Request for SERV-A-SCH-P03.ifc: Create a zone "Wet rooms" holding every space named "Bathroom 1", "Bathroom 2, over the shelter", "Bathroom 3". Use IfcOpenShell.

First a look at what the model holds.

```python
import ifcopenshell

model = ifcopenshell.open("SERV-A-SCH-P03.ifc")
print(model.schema)
seen = {}
for space in model.by_type("IfcSpace"):
    seen[space.LongName] = seen.get(space.LongName, 0) + 1
for name, count in sorted(seen.items(), key=str):
    print(count, "x", name)
print("zones:", [z.Name for z in model.by_type("IfcZone")][:20])
```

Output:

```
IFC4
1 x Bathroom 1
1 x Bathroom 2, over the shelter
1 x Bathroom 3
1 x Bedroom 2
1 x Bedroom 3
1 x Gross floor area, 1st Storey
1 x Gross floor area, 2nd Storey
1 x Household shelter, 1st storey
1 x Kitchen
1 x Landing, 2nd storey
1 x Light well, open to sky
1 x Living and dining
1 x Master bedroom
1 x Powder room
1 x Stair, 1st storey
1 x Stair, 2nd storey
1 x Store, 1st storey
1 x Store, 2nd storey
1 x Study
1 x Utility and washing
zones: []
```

```python
import ifcopenshell
import ifcopenshell.api.group
import ifcopenshell.api.root

model = ifcopenshell.open("SERV-A-SCH-P03.ifc")

names = {"Bathroom 1", "Bathroom 2, over the shelter", "Bathroom 3"}
spaces = [s for s in model.by_type("IfcSpace") if s.LongName in names]

zone = ifcopenshell.api.root.create_entity(model, ifc_class="IfcZone", name="Wet rooms")
ifcopenshell.api.group.assign_group(model, products=spaces, group=zone)
print(len(spaces), "spaces in", zone.Name)

model.write("SERV-A-SCH-P03_updated.ifc")
```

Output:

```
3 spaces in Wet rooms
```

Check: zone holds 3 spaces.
